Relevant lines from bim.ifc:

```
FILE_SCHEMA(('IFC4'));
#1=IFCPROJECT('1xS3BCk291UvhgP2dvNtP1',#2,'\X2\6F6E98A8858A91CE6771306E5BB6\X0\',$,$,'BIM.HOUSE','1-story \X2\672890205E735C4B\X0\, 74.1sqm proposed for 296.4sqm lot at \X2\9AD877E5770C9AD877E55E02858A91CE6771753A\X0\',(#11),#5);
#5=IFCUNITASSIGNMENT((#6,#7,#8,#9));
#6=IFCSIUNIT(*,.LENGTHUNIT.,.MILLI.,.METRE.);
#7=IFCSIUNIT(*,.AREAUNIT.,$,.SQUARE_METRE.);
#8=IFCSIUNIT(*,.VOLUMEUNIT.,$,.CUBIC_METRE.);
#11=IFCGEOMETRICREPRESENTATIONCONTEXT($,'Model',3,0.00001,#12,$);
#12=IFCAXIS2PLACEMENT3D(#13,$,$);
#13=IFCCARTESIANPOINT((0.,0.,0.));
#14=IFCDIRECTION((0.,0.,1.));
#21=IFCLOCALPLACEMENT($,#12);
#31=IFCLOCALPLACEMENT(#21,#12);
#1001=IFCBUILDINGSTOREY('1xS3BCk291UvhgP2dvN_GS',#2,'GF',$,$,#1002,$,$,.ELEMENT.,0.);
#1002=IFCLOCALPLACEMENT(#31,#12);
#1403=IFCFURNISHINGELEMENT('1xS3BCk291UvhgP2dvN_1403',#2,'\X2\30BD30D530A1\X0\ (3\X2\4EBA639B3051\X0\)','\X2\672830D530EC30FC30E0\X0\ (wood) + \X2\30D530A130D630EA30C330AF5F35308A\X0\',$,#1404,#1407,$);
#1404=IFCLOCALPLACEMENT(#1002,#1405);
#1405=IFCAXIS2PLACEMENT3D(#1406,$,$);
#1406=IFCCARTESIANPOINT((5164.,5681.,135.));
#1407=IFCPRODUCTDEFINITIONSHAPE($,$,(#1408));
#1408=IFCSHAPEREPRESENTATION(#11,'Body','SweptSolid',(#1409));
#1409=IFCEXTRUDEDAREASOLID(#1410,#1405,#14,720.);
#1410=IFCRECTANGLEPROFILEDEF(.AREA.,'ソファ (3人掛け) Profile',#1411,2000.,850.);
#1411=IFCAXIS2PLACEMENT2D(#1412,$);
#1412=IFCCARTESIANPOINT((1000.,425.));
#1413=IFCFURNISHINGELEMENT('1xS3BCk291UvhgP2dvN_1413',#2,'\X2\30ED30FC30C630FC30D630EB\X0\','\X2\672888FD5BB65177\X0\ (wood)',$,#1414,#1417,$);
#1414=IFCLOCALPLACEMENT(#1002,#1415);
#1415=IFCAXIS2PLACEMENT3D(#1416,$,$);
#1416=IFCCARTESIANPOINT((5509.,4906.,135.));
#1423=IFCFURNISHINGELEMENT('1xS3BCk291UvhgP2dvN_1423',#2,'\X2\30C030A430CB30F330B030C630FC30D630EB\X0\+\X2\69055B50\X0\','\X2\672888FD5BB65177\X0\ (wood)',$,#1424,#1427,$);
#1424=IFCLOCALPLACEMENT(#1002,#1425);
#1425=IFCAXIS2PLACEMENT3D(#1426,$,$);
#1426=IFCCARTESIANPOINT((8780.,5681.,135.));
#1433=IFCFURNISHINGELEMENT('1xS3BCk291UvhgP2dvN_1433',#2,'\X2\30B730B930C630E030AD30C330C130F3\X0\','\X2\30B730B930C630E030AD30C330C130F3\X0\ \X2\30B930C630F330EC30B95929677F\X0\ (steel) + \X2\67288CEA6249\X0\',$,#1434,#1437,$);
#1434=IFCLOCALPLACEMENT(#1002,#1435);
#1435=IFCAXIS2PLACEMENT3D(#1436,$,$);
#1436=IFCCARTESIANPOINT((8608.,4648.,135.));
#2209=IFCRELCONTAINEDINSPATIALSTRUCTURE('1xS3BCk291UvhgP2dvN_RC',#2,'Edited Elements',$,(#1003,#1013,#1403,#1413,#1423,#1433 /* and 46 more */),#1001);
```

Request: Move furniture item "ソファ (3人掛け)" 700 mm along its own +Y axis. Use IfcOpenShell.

```python
import ifcopenshell
import ifcopenshell.api.geometry
import ifcopenshell.util.placement

model = ifcopenshell.open("bim.ifc")

item = model.by_guid("1xS3BCk291UvhgP2dvN_1403")
matrix = ifcopenshell.util.placement.get_local_placement(item.ObjectPlacement)
matrix[:3, 3] += matrix[:3, 1] * 700.0
ifcopenshell.api.geometry.edit_object_placement(model, product=item, matrix=matrix, is_si=False)

print(ifcopenshell.util.placement.get_local_placement(item.ObjectPlacement).round(3) + 0.0)

model.write("bim_v2.ifc")
```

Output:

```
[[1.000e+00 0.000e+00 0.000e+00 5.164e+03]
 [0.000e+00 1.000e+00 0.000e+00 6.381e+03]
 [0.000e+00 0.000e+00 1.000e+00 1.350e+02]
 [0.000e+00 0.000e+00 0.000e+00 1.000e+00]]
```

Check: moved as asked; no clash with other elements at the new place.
